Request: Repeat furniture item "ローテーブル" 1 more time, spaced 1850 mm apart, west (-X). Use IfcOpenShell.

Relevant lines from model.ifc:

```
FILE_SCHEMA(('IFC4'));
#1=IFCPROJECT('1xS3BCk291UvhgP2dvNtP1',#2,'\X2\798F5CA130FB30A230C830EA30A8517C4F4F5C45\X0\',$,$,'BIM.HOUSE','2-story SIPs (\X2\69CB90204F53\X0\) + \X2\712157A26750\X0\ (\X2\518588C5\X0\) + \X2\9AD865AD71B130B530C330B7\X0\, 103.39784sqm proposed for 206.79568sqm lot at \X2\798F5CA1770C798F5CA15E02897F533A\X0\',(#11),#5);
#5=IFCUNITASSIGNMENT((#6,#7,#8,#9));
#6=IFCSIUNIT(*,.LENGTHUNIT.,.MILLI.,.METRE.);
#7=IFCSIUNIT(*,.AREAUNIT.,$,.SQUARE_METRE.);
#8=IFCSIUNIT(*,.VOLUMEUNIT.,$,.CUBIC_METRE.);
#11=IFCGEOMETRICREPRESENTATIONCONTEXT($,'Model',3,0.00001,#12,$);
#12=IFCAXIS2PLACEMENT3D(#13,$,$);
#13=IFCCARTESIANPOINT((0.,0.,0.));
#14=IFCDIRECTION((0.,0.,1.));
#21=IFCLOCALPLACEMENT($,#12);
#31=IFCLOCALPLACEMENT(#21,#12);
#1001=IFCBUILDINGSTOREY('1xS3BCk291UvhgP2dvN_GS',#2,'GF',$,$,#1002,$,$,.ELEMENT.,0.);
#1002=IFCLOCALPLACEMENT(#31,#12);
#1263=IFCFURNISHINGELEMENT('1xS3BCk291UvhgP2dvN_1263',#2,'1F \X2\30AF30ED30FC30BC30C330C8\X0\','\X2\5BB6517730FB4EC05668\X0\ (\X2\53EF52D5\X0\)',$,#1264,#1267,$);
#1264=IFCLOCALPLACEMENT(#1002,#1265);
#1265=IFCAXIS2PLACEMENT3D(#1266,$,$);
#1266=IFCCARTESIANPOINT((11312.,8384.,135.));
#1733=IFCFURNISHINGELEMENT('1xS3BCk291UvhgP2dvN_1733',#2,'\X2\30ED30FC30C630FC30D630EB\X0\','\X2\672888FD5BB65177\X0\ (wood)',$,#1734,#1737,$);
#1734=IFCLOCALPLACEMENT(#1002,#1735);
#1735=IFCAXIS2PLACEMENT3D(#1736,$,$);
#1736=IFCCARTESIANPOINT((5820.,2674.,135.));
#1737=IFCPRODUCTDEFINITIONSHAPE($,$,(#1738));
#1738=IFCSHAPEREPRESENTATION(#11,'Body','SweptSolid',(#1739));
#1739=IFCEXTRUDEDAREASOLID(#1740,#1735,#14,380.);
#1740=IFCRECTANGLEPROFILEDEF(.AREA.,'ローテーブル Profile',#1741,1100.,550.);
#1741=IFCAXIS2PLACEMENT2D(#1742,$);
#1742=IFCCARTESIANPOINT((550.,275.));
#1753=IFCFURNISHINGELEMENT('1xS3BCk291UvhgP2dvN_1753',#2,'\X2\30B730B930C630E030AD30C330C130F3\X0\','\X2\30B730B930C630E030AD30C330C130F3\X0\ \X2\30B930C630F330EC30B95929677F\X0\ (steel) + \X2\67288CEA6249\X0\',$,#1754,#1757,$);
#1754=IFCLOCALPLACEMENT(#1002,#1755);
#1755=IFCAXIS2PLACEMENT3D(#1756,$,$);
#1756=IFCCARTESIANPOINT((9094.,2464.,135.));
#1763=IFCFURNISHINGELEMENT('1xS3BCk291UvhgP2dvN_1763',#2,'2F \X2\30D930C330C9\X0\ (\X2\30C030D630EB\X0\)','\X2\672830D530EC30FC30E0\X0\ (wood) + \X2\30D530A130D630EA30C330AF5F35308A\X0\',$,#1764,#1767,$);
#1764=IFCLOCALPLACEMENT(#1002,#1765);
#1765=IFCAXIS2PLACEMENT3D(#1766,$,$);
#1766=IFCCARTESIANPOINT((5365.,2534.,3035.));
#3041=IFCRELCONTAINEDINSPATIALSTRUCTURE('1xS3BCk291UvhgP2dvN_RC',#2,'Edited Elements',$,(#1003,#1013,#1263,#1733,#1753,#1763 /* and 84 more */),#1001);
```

```python
import numpy as np
import ifcopenshell
import ifcopenshell.api.geometry
import ifcopenshell.api.root
import ifcopenshell.util.element
import ifcopenshell.util.placement
import ifcopenshell.util.unit

model = ifcopenshell.open("model.ifc")
unit_scale = ifcopenshell.util.unit.calculate_unit_scale(model)


def reuse_history(source, copy):
    """copy_class also copies each property set's owner history, people and application; keep the originals."""
    for rel in copy.IsDefinedBy:
        if rel.is_a("IfcRelDefinesByProperties") and (history := rel.RelatingPropertyDefinition.OwnerHistory):
            rel.RelatingPropertyDefinition.OwnerHistory = source.OwnerHistory
            ifcopenshell.util.element.remove_deep2(model, history)


source = model.by_id(1733)
base = ifcopenshell.util.placement.get_local_placement(source.ObjectPlacement)
step = np.array([-1.0, 0.0, 0.0]) * 1.85 / unit_scale

for i in range(1, 2):
    copy = ifcopenshell.api.root.copy_class(model, product=source)
    copy.Representation = ifcopenshell.util.element.copy_deep(
        model, source.Representation, exclude=["IfcGeometricRepresentationContext", "IfcRepresentationMap"]
    )
    reuse_history(source, copy)
    matrix = base.copy()
    matrix[:3, 3] += i * step
    print("added at", matrix[:3, 3].round(3) + 0.0)
    ifcopenshell.api.geometry.edit_object_placement(model, product=copy, matrix=matrix, is_si=False)

model.write("model_v2.ifc")
```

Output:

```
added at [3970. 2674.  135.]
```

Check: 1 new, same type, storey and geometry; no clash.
